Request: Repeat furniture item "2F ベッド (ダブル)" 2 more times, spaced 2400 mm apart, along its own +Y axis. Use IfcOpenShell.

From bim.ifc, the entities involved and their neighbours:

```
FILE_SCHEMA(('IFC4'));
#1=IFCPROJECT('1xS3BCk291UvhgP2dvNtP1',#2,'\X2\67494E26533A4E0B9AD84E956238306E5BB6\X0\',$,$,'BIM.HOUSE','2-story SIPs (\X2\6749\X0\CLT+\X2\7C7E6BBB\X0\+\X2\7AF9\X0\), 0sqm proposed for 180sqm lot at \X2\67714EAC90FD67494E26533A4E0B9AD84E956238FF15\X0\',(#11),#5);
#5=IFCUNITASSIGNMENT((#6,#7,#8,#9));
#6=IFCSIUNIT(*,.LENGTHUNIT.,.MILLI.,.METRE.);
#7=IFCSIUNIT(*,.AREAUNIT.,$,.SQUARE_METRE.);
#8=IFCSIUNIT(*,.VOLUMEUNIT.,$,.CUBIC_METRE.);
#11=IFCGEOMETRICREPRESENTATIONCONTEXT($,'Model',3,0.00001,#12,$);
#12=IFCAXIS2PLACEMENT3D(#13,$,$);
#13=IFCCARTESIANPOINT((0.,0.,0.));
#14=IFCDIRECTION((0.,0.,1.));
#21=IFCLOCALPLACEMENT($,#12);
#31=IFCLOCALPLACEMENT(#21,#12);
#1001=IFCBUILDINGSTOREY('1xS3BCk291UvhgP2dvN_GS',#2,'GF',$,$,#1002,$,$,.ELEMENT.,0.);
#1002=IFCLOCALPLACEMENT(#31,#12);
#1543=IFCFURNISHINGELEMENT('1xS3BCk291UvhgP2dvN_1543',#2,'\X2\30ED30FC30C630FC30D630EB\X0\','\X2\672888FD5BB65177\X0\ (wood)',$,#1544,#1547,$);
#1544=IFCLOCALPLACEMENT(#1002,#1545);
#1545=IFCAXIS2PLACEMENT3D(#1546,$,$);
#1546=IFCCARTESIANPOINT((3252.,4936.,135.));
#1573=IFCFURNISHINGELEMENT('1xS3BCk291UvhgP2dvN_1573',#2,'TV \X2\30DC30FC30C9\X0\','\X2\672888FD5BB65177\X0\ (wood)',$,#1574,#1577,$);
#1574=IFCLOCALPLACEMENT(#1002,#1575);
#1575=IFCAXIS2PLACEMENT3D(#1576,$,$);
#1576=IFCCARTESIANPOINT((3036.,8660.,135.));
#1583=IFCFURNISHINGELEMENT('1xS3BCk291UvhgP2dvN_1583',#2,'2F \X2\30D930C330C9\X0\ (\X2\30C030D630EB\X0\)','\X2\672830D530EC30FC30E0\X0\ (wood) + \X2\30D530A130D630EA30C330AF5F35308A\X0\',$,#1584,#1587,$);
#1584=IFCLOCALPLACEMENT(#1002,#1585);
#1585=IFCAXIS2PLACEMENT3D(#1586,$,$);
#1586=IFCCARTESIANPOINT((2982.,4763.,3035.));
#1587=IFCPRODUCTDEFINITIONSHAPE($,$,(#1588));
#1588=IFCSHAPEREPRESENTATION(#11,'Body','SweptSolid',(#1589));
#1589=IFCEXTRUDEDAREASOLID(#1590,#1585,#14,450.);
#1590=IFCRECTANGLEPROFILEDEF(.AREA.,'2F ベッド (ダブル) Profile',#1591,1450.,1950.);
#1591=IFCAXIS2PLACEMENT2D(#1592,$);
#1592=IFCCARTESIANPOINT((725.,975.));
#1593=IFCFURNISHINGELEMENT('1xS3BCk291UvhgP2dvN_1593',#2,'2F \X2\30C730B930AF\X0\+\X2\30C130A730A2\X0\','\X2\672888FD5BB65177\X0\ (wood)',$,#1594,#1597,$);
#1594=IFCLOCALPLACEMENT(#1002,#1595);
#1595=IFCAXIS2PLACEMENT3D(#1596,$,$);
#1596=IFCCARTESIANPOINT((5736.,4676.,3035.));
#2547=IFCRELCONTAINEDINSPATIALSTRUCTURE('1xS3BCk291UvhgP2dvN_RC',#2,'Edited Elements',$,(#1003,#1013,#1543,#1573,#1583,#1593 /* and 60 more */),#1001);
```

```python
import ifcopenshell
import ifcopenshell.api.geometry
import ifcopenshell.api.root
import ifcopenshell.util.element
import ifcopenshell.util.placement

model = ifcopenshell.open("bim.ifc")


def reuse_history(source, copy):
    """copy_class also copies each property set's owner history, people and application; keep the originals."""
    for rel in copy.IsDefinedBy:
        if rel.is_a("IfcRelDefinesByProperties") and (history := rel.RelatingPropertyDefinition.OwnerHistory):
            rel.RelatingPropertyDefinition.OwnerHistory = source.OwnerHistory
            ifcopenshell.util.element.remove_deep2(model, history)


source = model.by_guid("1xS3BCk291UvhgP2dvN_1583")
base = ifcopenshell.util.placement.get_local_placement(source.ObjectPlacement)
step = base[:3, 1] * 2400.0

for i in range(1, 3):
    copy = ifcopenshell.api.root.copy_class(model, product=source)
    copy.Representation = ifcopenshell.util.element.copy_deep(
        model, source.Representation, exclude=["IfcGeometricRepresentationContext", "IfcRepresentationMap"]
    )
    reuse_history(source, copy)
    matrix = base.copy()
    matrix[:3, 3] += i * step
    print("added at", matrix[:3, 3].round(3) + 0.0)
    ifcopenshell.api.geometry.edit_object_placement(model, product=copy, matrix=matrix, is_si=False)

model.write("bim_edited.ifc")
```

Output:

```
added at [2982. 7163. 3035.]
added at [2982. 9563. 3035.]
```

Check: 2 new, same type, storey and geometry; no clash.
